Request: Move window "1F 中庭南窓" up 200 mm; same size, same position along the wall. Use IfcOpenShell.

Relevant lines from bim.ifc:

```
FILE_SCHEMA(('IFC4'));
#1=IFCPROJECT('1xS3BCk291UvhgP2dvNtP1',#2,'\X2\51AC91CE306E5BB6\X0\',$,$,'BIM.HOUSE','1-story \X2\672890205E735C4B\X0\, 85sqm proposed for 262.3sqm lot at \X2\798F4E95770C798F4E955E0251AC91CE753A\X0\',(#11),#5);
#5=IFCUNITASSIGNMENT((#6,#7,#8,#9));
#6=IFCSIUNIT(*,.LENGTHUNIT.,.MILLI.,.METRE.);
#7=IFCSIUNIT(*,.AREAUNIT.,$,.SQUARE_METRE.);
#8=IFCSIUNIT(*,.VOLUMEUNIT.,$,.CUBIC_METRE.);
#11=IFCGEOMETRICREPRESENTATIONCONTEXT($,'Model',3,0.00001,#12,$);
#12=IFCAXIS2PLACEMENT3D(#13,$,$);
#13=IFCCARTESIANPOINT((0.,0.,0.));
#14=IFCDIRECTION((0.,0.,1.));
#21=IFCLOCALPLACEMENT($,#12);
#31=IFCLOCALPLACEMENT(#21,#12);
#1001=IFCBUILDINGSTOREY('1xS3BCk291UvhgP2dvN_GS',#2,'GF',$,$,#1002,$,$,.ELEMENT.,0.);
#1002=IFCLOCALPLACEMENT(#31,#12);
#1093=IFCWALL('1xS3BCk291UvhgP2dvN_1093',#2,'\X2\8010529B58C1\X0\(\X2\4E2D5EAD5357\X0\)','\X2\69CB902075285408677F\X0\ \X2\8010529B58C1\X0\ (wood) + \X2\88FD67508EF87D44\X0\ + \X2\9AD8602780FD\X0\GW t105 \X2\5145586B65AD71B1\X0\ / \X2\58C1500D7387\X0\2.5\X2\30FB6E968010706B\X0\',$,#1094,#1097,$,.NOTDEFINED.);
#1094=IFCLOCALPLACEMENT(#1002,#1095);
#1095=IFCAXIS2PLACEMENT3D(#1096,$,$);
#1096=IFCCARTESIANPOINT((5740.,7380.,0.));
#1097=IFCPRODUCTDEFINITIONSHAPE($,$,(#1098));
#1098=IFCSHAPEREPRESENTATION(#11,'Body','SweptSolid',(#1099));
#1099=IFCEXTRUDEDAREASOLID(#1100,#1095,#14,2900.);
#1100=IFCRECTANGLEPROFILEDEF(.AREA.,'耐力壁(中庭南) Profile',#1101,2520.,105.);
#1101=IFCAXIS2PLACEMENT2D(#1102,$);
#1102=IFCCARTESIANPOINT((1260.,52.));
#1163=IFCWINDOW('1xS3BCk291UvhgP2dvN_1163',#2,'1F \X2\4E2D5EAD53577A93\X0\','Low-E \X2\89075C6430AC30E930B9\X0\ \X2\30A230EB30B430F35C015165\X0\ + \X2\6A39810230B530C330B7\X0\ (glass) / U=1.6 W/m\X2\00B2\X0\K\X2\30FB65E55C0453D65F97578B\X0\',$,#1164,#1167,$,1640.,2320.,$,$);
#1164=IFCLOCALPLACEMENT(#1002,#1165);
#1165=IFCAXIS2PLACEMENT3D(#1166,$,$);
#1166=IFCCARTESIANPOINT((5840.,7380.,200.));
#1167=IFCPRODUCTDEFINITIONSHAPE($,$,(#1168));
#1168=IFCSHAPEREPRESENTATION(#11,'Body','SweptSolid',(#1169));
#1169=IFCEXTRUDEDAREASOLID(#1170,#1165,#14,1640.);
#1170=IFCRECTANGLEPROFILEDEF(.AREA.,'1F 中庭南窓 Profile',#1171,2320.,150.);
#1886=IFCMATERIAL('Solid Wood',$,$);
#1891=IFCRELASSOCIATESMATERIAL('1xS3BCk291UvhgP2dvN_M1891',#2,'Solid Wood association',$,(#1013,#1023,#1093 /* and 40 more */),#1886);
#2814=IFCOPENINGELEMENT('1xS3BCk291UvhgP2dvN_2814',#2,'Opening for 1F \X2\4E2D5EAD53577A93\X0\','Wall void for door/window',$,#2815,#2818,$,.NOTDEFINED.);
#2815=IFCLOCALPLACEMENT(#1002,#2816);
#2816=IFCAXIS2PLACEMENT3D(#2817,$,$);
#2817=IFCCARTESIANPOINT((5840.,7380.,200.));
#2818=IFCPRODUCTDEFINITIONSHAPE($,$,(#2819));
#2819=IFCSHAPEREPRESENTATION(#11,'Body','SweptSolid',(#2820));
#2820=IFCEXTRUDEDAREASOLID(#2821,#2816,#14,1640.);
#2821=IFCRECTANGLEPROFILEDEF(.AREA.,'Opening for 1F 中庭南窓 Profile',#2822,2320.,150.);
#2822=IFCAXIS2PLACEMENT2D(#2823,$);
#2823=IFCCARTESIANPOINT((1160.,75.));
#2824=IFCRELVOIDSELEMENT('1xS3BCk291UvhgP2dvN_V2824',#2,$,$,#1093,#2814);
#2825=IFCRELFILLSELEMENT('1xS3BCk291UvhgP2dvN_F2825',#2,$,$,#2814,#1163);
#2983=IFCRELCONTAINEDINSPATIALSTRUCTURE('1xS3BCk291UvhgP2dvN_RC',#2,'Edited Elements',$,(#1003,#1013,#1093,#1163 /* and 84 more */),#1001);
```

```python
import numpy as np
import ifcopenshell
import ifcopenshell.api.geometry
import ifcopenshell.util.placement
import ifcopenshell.util.unit

model = ifcopenshell.open("bim.ifc")
unit_scale = ifcopenshell.util.unit.calculate_unit_scale(model)

window = model.by_guid("1xS3BCk291UvhgP2dvN_1163")
opening = window.FillsVoids[0].RelatingOpeningElement
dz = 0.2 / unit_scale

shift = np.array([0.0, 0.0, dz])
# The window is not placed relative to its opening, so move both.
for product in (opening, window):
    matrix = ifcopenshell.util.placement.get_local_placement(product.ObjectPlacement)
    matrix[:3, 3] += shift
    ifcopenshell.api.geometry.edit_object_placement(model, product=product, matrix=matrix, is_si=False)

print(f"moved by {dz * unit_scale:+.3f} m")

model.write("bim_updated.ifc")
```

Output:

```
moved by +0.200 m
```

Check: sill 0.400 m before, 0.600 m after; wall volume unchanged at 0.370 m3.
